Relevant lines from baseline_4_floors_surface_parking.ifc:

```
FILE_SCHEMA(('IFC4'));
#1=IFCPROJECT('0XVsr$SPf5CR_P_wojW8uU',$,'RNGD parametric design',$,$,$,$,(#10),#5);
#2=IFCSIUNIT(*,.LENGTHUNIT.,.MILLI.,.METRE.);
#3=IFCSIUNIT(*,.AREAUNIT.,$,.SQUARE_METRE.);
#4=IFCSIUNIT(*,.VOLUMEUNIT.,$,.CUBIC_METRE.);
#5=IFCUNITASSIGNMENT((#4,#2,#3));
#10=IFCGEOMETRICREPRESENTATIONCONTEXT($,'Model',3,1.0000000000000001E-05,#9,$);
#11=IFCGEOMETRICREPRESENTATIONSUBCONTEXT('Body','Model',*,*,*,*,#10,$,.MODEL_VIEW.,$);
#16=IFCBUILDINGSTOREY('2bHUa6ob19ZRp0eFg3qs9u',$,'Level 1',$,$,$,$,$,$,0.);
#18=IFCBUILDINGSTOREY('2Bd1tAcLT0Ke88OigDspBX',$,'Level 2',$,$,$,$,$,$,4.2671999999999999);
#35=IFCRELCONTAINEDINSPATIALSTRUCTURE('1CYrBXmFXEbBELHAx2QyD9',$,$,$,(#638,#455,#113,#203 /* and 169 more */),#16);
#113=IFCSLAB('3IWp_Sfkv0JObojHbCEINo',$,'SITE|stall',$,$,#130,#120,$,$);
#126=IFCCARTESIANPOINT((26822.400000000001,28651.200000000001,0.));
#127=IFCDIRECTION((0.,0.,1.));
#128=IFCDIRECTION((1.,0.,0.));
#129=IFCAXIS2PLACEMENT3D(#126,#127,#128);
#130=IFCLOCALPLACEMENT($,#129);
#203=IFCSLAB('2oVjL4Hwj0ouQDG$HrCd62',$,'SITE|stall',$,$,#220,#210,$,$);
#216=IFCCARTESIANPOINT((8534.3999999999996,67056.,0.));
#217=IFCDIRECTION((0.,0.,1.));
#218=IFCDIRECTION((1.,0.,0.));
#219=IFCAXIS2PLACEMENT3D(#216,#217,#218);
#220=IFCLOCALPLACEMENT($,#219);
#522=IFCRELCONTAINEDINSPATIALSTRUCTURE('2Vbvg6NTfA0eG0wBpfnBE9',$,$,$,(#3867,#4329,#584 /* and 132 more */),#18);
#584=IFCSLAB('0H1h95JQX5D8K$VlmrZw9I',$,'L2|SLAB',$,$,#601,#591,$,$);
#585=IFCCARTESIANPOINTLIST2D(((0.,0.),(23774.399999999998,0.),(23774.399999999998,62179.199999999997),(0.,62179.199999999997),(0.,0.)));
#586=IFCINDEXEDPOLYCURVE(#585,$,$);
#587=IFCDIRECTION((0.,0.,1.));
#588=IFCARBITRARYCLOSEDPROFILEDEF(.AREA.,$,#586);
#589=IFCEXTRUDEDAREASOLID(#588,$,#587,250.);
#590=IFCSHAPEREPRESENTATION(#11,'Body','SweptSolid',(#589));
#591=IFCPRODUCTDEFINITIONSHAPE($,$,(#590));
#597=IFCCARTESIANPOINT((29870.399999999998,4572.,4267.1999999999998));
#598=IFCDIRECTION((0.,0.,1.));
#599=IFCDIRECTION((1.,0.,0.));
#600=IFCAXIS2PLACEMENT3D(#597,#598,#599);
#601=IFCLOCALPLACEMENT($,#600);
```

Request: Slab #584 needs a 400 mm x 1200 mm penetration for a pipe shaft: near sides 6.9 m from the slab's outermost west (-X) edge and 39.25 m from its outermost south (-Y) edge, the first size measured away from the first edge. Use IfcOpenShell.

```python
import numpy as np
import ifcopenshell
import ifcopenshell.api.feature
import ifcopenshell.api.geometry
import ifcopenshell.api.root
import ifcopenshell.geom
import ifcopenshell.util.placement
import ifcopenshell.util.representation
import ifcopenshell.util.shape
import ifcopenshell.util.unit

model = ifcopenshell.open("baseline_4_floors_surface_parking.ifc")
unit_scale = ifcopenshell.util.unit.calculate_unit_scale(model)
settings = ifcopenshell.geom.settings()


def volume(element):
    """Net volume in cubic metres, openings subtracted."""
    shape = ifcopenshell.geom.create_shape(settings, element)
    return ifcopenshell.util.shape.get_volume(shape.geometry)


slab = model.by_id(584)
before = volume(slab)

# Extent in the slab's own axes, in metres. The edges named are its -X and -Y sides.
slab_shape = ifcopenshell.geom.create_shape(settings, slab)
vertices = ifcopenshell.util.shape.get_vertices(slab_shape.geometry)
x_min, y_min, bottom = vertices.min(axis=0)
top = vertices[:, 2].max()

opening = ifcopenshell.api.root.create_entity(model, ifc_class="IfcOpeningElement", name="Pipe shaft opening", predefined_type="OPENING")
context = ifcopenshell.util.representation.get_context(model, "Model", "Body", "MODEL_VIEW")
width, depth = 0.4, 1.2
outline = [(0.0, 0.0), (width, 0.0), (width, depth), (0.0, depth), (0.0, 0.0)]
# Overshoot both faces by 50 mm so the cut is clean.
shape = ifcopenshell.api.geometry.add_slab_representation(
    model, context=context, depth=top - bottom + 0.1, polyline=outline
)
ifcopenshell.api.geometry.assign_representation(model, product=opening, representation=shape)

matrix = ifcopenshell.util.placement.get_local_placement(slab.ObjectPlacement)
matrix[:, 3] = matrix @ np.append(np.array([x_min + 6.9, y_min + 39.25, bottom - 0.05]) / unit_scale, 1.0)
ifcopenshell.api.geometry.edit_object_placement(model, product=opening, matrix=matrix, is_si=False)
ifcopenshell.api.feature.add_feature(model, feature=opening, element=slab)

after = volume(slab)

print(f"slab volume {before:.3f} -> {after:.3f} m3")

model.write("baseline_4_floors_surface_parking_updated.ifc")
```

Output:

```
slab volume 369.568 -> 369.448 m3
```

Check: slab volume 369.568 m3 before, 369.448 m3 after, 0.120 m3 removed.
